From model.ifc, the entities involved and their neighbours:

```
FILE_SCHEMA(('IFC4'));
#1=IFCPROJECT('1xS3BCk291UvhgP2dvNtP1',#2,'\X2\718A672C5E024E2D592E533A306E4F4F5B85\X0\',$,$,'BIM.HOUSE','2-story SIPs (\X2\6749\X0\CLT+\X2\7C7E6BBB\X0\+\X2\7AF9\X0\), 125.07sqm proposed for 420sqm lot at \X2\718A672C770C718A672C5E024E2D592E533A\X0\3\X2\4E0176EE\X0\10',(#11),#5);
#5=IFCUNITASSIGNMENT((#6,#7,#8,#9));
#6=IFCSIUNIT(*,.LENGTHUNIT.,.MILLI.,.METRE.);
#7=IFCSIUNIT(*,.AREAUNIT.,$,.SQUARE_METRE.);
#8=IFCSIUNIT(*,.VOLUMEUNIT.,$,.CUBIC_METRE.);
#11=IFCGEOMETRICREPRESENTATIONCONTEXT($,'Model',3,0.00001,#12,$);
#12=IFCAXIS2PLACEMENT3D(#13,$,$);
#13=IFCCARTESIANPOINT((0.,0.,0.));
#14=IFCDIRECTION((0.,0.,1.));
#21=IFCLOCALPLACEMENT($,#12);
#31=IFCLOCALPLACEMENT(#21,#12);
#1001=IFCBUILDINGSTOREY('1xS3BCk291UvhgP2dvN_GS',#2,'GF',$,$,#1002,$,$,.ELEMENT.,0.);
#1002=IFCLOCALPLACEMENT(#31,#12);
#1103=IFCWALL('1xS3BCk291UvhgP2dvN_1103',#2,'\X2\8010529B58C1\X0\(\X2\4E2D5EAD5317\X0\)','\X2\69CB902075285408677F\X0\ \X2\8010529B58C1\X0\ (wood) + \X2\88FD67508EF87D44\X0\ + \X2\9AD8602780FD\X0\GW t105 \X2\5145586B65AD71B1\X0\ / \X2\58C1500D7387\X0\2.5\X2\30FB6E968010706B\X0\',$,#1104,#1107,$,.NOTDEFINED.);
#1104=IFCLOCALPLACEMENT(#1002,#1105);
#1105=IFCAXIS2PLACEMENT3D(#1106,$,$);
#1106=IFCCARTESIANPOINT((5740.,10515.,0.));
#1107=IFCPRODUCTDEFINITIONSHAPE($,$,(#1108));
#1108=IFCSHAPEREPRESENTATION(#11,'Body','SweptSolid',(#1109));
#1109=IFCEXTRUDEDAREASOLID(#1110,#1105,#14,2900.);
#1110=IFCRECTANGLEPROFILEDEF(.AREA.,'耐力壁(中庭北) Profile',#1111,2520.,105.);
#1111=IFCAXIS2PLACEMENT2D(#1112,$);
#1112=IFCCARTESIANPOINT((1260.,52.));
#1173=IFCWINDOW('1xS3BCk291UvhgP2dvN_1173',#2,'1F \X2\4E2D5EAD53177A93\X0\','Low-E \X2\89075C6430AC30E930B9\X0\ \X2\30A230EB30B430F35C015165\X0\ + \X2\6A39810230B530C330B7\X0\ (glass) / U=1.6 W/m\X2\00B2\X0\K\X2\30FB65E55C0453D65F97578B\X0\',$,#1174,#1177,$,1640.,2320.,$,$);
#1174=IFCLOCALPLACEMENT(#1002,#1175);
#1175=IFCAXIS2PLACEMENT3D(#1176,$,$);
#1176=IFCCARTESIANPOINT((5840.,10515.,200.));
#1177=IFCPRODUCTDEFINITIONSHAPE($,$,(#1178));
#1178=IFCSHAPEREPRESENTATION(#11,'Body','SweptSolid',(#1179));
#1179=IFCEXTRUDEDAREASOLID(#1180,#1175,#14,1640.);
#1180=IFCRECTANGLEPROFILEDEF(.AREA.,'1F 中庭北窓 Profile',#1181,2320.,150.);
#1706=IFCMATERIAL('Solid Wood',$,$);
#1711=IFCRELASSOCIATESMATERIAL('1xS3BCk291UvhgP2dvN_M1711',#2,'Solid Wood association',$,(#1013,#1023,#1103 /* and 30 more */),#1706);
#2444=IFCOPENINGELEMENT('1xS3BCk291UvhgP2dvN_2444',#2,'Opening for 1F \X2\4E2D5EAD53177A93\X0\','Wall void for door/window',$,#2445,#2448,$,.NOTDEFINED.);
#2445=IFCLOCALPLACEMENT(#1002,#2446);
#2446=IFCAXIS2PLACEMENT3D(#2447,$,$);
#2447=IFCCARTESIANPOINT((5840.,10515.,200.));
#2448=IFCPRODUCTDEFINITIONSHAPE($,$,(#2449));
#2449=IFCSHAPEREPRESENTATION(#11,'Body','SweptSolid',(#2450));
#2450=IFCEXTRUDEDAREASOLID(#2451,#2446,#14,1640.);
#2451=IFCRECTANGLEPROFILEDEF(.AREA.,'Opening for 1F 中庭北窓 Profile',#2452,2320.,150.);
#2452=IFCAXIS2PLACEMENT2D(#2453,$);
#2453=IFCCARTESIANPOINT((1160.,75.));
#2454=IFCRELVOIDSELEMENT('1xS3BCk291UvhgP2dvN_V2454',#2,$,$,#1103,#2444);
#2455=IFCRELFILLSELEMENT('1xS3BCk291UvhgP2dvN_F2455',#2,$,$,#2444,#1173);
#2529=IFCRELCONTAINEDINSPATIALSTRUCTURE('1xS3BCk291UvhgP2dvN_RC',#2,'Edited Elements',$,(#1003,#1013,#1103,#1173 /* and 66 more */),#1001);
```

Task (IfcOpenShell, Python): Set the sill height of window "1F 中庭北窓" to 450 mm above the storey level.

```python
import numpy as np
import ifcopenshell
import ifcopenshell.api.geometry
import ifcopenshell.geom
import ifcopenshell.util.element
import ifcopenshell.util.placement
import ifcopenshell.util.shape
import ifcopenshell.util.unit

model = ifcopenshell.open("model.ifc")
unit_scale = ifcopenshell.util.unit.calculate_unit_scale(model)

window = model.by_guid("1xS3BCk291UvhgP2dvN_1173")
opening = window.FillsVoids[0].RelatingOpeningElement
storey = ifcopenshell.util.element.get_container(window, ifc_class="IfcBuildingStorey")
level = ifcopenshell.util.placement.get_local_placement(storey.ObjectPlacement)[2, 3]

# The opening's origin need not be at the sill, so measure its lowest point.
shape = ifcopenshell.geom.create_shape(ifcopenshell.geom.settings(), opening)
bottom = ifcopenshell.util.shape.get_shape_bottom_elevation(shape, shape.geometry) / unit_scale
dz = level + 0.45 / unit_scale - bottom

shift = np.array([0.0, 0.0, dz])
# The window is not placed relative to its opening, so move both.
for product in (opening, window):
    matrix = ifcopenshell.util.placement.get_local_placement(product.ObjectPlacement)
    matrix[:3, 3] += shift
    ifcopenshell.api.geometry.edit_object_placement(model, product=product, matrix=matrix, is_si=False)

print(f"moved by {dz * unit_scale:+.3f} m")

model.write("model_rev.ifc")
```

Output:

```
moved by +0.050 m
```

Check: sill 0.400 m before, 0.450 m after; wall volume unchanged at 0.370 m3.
